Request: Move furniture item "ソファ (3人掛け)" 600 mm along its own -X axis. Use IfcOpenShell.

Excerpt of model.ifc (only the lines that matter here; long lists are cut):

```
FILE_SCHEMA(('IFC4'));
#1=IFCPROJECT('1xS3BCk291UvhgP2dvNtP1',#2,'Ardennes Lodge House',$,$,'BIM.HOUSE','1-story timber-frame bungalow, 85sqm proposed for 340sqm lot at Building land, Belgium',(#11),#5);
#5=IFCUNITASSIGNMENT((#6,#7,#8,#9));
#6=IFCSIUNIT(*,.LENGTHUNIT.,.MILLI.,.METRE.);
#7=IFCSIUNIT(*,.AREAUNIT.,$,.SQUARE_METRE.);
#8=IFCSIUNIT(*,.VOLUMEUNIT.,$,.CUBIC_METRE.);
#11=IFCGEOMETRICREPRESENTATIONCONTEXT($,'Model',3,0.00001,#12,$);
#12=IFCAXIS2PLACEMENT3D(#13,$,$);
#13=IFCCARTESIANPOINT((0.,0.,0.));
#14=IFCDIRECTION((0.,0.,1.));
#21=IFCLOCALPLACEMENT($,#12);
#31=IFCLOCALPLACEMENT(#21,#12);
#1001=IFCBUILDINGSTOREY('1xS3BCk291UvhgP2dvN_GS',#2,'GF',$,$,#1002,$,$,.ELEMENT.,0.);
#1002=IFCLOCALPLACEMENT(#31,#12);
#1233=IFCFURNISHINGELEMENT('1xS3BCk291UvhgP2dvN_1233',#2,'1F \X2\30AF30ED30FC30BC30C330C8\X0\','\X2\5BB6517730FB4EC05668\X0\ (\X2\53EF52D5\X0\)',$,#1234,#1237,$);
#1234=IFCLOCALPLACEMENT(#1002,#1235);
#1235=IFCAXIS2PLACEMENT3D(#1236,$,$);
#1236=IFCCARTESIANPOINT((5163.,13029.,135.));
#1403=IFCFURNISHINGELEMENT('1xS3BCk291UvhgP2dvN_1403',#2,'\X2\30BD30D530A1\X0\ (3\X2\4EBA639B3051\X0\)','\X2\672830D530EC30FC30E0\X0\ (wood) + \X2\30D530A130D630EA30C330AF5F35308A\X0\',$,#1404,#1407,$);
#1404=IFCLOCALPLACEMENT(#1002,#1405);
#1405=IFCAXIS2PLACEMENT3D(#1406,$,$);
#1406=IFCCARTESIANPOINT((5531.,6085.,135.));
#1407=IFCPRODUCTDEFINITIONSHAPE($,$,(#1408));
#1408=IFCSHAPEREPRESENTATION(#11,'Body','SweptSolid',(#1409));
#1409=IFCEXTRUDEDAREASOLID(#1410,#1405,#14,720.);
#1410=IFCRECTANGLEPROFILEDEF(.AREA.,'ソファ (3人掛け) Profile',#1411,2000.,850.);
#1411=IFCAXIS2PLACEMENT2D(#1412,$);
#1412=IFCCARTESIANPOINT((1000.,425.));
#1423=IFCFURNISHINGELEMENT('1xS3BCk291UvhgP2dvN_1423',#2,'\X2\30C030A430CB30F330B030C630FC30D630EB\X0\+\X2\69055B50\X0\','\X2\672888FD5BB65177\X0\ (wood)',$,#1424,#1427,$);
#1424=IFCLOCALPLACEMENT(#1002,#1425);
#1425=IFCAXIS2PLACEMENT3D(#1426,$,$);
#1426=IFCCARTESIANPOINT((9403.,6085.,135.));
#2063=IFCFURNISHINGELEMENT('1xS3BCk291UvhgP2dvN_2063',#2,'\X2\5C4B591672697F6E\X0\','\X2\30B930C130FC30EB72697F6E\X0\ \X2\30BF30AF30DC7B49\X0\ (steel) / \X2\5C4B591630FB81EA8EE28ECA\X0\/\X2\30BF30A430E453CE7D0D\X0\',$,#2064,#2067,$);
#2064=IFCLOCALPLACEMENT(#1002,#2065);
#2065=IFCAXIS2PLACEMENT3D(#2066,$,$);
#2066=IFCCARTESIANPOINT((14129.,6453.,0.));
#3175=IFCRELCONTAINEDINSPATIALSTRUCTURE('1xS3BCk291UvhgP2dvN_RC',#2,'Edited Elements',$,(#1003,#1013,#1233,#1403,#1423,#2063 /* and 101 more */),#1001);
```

```python
import ifcopenshell
import ifcopenshell.api.geometry
import ifcopenshell.util.placement

model = ifcopenshell.open("model.ifc")

item = model.by_guid("1xS3BCk291UvhgP2dvN_1403")
matrix = ifcopenshell.util.placement.get_local_placement(item.ObjectPlacement)
matrix[:3, 3] -= matrix[:3, 0] * 600.0
ifcopenshell.api.geometry.edit_object_placement(model, product=item, matrix=matrix, is_si=False)

print(ifcopenshell.util.placement.get_local_placement(item.ObjectPlacement).round(3) + 0.0)

model.write("model_edited.ifc")
```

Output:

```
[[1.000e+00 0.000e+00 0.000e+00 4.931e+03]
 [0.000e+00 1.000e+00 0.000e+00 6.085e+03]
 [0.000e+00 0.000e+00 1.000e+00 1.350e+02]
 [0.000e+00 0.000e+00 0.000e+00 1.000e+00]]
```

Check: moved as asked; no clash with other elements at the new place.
